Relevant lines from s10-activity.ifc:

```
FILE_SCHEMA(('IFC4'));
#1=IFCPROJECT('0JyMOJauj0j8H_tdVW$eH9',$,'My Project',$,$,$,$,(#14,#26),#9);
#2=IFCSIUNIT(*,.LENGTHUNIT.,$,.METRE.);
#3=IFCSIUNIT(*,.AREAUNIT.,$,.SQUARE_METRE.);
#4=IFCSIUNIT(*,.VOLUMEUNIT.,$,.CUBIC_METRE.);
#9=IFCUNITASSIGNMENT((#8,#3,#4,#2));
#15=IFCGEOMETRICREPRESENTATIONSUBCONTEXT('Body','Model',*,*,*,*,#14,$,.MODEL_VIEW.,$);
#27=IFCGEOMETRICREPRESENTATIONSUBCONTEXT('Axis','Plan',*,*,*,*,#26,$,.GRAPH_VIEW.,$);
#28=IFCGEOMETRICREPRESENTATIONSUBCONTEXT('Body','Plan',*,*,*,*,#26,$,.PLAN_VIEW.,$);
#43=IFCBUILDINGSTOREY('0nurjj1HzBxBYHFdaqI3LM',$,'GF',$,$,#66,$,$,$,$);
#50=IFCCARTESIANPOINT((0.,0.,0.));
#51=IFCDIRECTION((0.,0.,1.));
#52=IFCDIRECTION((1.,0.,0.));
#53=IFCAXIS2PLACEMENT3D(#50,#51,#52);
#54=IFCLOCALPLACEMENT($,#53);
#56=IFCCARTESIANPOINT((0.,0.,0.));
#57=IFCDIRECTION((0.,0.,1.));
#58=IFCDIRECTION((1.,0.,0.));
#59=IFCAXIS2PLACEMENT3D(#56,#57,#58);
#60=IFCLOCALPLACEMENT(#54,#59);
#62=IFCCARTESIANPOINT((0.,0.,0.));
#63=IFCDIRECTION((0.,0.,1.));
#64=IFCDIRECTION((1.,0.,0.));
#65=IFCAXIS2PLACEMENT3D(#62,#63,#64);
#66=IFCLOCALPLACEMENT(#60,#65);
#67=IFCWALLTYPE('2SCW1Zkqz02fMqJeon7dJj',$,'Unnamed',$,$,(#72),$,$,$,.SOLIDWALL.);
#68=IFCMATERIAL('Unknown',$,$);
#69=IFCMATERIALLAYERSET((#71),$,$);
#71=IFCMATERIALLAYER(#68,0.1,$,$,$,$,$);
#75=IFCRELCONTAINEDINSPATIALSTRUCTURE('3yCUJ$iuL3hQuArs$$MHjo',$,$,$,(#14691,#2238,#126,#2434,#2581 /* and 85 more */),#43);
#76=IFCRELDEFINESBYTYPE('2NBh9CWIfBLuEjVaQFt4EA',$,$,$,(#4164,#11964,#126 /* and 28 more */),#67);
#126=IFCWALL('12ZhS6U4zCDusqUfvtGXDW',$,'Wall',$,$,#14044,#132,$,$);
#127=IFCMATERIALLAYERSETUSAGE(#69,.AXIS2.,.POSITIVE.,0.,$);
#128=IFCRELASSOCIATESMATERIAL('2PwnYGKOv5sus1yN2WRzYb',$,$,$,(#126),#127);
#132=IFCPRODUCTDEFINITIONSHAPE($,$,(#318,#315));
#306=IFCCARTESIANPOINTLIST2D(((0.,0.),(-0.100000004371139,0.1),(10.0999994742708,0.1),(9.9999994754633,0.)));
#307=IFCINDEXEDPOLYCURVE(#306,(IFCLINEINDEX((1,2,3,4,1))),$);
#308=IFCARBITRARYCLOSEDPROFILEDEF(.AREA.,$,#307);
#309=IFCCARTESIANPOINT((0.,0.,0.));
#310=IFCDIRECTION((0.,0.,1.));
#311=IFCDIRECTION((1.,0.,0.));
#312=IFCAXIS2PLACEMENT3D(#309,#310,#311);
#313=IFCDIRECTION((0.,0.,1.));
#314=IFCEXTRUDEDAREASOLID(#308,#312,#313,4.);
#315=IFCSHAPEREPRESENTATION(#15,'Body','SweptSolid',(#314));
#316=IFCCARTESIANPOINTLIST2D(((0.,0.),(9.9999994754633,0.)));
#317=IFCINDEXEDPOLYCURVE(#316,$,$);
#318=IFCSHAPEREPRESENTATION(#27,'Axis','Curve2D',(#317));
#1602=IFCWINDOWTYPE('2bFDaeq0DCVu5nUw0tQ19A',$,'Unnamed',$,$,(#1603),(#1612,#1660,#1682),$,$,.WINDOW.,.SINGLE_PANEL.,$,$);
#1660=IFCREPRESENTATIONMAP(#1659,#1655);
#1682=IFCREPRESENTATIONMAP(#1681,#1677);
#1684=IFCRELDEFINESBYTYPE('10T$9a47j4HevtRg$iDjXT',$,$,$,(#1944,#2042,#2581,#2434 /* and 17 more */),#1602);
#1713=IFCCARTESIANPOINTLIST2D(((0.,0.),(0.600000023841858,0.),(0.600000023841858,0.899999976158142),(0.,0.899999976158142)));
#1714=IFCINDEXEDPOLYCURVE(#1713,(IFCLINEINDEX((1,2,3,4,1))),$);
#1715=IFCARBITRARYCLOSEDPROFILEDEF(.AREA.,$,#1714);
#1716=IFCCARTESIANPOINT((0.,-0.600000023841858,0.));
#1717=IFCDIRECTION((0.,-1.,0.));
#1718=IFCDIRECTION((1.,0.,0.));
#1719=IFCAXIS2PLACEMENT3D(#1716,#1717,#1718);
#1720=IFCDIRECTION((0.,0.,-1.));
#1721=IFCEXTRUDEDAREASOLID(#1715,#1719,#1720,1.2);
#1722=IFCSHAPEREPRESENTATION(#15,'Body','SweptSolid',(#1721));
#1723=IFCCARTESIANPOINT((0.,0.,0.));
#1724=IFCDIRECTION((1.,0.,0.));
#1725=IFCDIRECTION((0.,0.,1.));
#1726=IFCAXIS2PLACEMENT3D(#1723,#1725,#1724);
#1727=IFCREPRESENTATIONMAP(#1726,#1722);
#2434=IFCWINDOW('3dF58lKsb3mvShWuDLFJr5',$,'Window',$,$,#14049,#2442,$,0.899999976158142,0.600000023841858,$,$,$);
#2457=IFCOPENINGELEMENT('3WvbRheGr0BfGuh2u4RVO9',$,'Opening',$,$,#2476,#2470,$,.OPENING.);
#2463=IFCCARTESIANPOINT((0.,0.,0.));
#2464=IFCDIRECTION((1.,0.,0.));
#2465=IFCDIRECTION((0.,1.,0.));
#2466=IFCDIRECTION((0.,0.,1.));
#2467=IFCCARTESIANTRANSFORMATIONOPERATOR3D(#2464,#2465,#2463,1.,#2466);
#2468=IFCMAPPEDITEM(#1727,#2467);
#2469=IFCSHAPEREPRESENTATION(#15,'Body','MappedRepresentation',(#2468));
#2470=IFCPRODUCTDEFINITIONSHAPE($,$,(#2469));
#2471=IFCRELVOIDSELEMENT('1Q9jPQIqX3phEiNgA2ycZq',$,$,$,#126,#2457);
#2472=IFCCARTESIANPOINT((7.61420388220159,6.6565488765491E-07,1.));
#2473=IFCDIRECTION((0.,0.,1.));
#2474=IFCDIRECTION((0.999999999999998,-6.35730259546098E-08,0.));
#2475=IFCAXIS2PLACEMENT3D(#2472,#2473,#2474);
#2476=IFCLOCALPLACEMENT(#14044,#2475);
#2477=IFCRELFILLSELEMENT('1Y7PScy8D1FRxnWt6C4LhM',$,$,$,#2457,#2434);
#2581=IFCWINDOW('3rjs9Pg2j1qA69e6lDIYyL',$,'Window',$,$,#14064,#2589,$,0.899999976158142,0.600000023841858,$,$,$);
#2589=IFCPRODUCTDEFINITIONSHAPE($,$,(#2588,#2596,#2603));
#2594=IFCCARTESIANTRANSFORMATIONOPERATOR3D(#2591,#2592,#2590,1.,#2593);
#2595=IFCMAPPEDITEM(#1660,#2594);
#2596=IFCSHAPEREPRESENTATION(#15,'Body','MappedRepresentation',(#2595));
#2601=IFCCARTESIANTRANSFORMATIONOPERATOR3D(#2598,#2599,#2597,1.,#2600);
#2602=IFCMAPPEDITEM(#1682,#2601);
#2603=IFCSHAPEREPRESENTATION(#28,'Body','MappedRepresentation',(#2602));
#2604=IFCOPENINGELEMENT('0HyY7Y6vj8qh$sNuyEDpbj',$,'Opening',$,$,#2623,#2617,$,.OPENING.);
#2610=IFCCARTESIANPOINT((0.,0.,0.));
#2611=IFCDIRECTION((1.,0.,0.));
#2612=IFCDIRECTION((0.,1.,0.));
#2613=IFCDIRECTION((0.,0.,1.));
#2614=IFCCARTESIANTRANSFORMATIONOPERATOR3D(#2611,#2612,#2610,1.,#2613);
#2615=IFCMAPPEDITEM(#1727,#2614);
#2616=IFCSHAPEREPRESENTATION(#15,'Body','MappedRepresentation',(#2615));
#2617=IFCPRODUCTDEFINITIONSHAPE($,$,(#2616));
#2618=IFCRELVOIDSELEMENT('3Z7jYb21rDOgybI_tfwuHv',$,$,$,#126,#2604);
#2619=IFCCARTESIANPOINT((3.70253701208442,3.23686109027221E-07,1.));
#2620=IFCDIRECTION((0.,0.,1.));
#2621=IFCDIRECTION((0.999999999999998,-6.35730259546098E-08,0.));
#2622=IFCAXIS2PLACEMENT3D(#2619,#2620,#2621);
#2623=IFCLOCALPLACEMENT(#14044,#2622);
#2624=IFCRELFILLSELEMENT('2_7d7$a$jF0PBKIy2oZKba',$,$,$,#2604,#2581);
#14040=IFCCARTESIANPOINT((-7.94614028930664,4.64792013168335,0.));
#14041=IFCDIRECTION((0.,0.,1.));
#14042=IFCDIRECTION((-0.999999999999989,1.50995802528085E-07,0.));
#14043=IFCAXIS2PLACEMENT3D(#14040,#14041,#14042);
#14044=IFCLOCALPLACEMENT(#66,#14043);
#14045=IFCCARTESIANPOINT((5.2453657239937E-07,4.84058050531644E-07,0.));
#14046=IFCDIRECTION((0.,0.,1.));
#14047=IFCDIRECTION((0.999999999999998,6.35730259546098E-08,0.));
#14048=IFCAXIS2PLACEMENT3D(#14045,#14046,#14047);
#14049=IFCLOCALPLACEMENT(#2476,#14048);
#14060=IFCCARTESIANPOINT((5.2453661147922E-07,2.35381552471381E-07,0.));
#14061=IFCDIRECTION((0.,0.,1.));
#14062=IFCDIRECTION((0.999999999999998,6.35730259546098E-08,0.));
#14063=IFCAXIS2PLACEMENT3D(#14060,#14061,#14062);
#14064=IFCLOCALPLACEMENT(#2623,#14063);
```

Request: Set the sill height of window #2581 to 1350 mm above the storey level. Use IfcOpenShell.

```python
import numpy as np
import ifcopenshell
import ifcopenshell.api.geometry
import ifcopenshell.geom
import ifcopenshell.util.element
import ifcopenshell.util.placement
import ifcopenshell.util.shape
import ifcopenshell.util.unit

model = ifcopenshell.open("s10-activity.ifc")
unit_scale = ifcopenshell.util.unit.calculate_unit_scale(model)

window = model.by_guid("3rjs9Pg2j1qA69e6lDIYyL")
opening = window.FillsVoids[0].RelatingOpeningElement
storey = ifcopenshell.util.element.get_container(window, ifc_class="IfcBuildingStorey")
level = ifcopenshell.util.placement.get_local_placement(storey.ObjectPlacement)[2, 3]

# The opening's origin need not be at the sill, so measure its lowest point.
shape = ifcopenshell.geom.create_shape(ifcopenshell.geom.settings(), opening)
bottom = ifcopenshell.util.shape.get_shape_bottom_elevation(shape, shape.geometry) / unit_scale
dz = level + 1.35 / unit_scale - bottom

shift = np.array([0.0, 0.0, dz])
# The window is placed relative to its opening, so it follows when the opening moves.
matrix = ifcopenshell.util.placement.get_local_placement(opening.ObjectPlacement)
matrix[:3, 3] += shift
ifcopenshell.api.geometry.edit_object_placement(
    model, product=opening, matrix=matrix, is_si=False, should_transform_children=True
)

print(f"moved by {dz * unit_scale:+.3f} m")

model.write("s10-activity-out.ifc")
```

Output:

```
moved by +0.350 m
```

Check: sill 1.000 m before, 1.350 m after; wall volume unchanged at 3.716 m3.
